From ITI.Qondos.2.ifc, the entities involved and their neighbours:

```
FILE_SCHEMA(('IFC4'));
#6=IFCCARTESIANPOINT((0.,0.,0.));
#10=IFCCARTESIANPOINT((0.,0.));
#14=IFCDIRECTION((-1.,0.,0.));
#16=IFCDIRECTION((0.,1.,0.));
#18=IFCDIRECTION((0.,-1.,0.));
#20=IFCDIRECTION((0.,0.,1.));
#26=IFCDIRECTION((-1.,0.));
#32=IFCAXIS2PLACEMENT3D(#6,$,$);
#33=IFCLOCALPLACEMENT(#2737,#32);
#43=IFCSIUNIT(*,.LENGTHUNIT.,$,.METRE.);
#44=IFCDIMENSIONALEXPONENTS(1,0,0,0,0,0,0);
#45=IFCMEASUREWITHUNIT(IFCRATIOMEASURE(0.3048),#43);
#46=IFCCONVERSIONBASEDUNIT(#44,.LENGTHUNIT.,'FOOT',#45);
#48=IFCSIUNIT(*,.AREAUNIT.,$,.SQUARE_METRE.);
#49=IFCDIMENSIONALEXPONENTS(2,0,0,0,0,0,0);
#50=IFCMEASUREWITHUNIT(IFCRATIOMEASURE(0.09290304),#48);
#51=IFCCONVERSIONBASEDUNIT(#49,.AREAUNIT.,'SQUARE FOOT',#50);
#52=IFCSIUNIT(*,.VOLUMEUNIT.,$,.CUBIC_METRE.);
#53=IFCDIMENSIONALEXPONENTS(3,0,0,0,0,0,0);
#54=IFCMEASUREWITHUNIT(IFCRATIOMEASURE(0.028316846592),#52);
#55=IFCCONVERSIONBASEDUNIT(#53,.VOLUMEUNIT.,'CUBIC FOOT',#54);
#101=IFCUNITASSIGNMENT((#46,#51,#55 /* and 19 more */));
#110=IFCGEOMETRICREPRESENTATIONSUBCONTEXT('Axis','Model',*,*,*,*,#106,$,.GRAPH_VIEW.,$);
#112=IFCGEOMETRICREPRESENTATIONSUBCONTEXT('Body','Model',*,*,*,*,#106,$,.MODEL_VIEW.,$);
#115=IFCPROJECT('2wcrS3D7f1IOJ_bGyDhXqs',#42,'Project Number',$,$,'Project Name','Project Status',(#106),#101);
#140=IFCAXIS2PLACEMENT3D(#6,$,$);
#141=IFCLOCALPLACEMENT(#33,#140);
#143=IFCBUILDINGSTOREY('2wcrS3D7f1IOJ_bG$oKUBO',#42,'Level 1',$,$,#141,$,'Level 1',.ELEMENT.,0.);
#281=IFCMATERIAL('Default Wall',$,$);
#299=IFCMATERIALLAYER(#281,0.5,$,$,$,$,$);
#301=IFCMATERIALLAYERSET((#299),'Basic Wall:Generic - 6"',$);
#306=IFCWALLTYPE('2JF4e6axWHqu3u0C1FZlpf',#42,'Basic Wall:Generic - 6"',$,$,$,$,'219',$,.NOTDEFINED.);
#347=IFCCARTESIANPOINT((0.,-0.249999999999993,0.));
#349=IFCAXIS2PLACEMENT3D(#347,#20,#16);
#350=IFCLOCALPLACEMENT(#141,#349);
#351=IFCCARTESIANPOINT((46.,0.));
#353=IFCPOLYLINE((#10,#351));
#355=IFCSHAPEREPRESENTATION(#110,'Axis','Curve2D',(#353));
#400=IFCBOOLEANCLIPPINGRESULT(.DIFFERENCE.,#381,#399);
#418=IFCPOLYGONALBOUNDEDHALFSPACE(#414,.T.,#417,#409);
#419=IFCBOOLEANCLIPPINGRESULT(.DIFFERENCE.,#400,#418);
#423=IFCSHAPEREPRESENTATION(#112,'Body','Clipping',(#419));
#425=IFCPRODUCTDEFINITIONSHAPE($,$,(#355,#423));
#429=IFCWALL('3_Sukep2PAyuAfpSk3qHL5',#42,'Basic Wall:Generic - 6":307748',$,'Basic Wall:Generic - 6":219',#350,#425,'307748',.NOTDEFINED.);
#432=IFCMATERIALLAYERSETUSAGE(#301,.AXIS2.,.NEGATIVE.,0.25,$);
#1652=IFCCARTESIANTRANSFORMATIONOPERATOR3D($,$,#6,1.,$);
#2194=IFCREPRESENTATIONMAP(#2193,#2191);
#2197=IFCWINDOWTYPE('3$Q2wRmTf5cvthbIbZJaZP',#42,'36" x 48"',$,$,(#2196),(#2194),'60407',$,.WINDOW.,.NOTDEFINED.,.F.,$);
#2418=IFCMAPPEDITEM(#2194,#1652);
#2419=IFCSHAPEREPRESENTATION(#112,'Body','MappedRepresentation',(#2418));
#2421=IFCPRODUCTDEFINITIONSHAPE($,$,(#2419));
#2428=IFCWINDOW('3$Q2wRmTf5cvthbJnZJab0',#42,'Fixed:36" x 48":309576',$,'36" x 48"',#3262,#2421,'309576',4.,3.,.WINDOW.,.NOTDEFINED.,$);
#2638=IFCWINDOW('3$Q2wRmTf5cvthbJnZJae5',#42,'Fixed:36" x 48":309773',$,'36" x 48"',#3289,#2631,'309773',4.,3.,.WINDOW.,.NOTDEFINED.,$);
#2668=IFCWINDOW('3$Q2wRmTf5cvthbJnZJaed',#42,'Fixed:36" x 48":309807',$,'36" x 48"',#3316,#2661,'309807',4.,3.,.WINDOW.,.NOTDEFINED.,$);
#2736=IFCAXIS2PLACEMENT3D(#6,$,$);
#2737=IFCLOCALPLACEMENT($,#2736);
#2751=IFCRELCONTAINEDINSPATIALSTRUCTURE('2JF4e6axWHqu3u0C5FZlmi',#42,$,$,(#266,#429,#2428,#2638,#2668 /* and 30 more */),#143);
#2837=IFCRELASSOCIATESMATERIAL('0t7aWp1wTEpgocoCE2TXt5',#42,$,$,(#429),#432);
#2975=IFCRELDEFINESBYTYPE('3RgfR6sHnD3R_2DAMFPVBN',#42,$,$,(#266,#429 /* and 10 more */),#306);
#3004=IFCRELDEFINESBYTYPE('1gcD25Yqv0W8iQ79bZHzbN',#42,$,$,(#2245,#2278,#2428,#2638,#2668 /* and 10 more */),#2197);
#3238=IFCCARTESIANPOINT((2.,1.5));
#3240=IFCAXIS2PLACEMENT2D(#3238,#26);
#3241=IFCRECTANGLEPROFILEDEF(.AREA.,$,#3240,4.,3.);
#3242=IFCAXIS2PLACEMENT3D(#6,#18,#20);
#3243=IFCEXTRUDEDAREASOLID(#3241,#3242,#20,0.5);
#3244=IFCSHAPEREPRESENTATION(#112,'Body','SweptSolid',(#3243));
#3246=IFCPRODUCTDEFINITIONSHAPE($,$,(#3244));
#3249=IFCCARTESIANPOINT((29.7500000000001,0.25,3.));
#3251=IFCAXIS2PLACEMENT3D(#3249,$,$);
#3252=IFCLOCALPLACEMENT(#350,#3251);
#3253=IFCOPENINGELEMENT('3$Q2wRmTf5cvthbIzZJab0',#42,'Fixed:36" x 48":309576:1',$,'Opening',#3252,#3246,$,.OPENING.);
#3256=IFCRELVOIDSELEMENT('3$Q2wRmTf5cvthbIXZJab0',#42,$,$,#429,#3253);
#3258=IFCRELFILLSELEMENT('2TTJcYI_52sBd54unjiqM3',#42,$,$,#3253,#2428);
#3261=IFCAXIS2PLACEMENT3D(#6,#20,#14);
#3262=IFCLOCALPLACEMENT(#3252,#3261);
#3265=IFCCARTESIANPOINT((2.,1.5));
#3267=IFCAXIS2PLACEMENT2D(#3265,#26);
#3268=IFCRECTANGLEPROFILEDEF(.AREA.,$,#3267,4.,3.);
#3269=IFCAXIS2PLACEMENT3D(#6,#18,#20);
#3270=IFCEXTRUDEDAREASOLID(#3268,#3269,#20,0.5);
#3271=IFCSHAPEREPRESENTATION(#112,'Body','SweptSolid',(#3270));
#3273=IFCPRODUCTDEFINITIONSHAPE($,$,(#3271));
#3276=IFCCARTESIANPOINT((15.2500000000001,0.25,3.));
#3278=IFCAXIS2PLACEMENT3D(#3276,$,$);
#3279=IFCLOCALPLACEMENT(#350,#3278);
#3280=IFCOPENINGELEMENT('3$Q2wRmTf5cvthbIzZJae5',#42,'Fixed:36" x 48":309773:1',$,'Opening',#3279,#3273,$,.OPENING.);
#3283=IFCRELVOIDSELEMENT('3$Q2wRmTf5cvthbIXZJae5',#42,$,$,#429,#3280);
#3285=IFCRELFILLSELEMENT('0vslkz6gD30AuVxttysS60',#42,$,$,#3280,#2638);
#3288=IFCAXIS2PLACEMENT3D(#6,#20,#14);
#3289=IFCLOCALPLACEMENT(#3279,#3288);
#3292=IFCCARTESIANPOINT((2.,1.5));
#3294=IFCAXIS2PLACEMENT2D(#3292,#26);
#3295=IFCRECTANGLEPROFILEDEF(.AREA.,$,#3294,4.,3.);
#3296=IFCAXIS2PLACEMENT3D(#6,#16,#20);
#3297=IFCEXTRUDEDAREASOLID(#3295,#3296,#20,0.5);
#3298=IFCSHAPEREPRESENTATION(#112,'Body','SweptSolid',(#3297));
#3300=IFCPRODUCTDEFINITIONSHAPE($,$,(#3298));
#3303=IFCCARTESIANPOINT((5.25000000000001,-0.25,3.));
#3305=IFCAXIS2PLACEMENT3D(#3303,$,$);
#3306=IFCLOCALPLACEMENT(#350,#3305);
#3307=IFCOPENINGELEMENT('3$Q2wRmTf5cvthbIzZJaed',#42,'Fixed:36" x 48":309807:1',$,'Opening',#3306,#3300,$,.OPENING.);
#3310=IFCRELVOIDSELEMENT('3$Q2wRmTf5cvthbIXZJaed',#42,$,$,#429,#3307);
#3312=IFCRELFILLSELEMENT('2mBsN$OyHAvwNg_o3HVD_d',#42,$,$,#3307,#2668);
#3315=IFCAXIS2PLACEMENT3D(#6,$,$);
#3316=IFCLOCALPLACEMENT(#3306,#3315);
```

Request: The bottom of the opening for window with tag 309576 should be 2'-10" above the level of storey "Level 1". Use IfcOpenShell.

```python
import numpy as np
import ifcopenshell
import ifcopenshell.api.geometry
import ifcopenshell.geom
import ifcopenshell.util.element
import ifcopenshell.util.placement
import ifcopenshell.util.shape
import ifcopenshell.util.unit

model = ifcopenshell.open("ITI.Qondos.2.ifc")
unit_scale = ifcopenshell.util.unit.calculate_unit_scale(model)

window = model.by_guid("3$Q2wRmTf5cvthbJnZJab0")
opening = window.FillsVoids[0].RelatingOpeningElement
storey = ifcopenshell.util.element.get_container(window, ifc_class="IfcBuildingStorey")
level = ifcopenshell.util.placement.get_local_placement(storey.ObjectPlacement)[2, 3]

# The opening's origin need not be at the sill, so measure its lowest point.
shape = ifcopenshell.geom.create_shape(ifcopenshell.geom.settings(), opening)
bottom = ifcopenshell.util.shape.get_shape_bottom_elevation(shape, shape.geometry) / unit_scale
dz = level + 34 * 0.0254 / unit_scale - bottom

shift = np.array([0.0, 0.0, dz])
# The window is placed relative to its opening, so it follows when the opening moves.
matrix = ifcopenshell.util.placement.get_local_placement(opening.ObjectPlacement)
matrix[:3, 3] += shift
ifcopenshell.api.geometry.edit_object_placement(
    model, product=opening, matrix=matrix, is_si=False, should_transform_children=True
)

print(f"moved by {dz * unit_scale:+.3f} m")

model.write("ITI.Qondos.2_updated.ifc")
```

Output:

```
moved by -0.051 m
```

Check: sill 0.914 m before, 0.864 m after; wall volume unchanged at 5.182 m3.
